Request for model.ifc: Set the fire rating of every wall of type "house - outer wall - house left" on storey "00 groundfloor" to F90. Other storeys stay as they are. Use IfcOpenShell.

First a look at what the model holds.

```python
import ifcopenshell
import ifcopenshell.util.element

model = ifcopenshell.open("model.ifc")
print(model.schema)
storey = next(s for s in model.by_type("IfcBuildingStorey") if s.Name == "00 groundfloor")
walls = [e for e in ifcopenshell.util.element.get_decomposition(storey) if e.is_a("IfcWall")]
seen = {}
for e in walls:
    element_type = ifcopenshell.util.element.get_type(e)
    key = (element_type.Name if element_type != e and element_type else None, ifcopenshell.util.element.get_pset(e, "Pset_WallCommon", "FireRating"))
    seen[key] = seen.get(key, 0) + 1
for (name, value), count in sorted(seen.items(), key=str):
    print(count, "x", name, "|", value)
```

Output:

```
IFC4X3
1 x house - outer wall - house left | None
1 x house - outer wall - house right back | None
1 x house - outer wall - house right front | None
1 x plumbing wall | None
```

```python
import ifcopenshell
import ifcopenshell.api.pset
import ifcopenshell.util.element

model = ifcopenshell.open("model.ifc")

storey = next(s for s in model.by_type("IfcBuildingStorey") if s.Name == "00 groundfloor")
walls = [e for e in ifcopenshell.util.element.get_decomposition(storey) if e.is_a("IfcWall")]

count = 0
for e in walls:
    element_type = ifcopenshell.util.element.get_type(e)
    if element_type in (None, e) or element_type.Name != "house - outer wall - house left":
        continue
    # add_pset returns the element's existing set when there is one.
    pset = ifcopenshell.api.pset.add_pset(model, product=e, name="Pset_WallCommon")
    ifcopenshell.api.pset.edit_pset(model, pset=pset, properties={"FireRating": "F90"})
    count += 1

print(count, "walls updated")

model.write("model_updated.ifc")
```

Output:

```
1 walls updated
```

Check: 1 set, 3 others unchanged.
